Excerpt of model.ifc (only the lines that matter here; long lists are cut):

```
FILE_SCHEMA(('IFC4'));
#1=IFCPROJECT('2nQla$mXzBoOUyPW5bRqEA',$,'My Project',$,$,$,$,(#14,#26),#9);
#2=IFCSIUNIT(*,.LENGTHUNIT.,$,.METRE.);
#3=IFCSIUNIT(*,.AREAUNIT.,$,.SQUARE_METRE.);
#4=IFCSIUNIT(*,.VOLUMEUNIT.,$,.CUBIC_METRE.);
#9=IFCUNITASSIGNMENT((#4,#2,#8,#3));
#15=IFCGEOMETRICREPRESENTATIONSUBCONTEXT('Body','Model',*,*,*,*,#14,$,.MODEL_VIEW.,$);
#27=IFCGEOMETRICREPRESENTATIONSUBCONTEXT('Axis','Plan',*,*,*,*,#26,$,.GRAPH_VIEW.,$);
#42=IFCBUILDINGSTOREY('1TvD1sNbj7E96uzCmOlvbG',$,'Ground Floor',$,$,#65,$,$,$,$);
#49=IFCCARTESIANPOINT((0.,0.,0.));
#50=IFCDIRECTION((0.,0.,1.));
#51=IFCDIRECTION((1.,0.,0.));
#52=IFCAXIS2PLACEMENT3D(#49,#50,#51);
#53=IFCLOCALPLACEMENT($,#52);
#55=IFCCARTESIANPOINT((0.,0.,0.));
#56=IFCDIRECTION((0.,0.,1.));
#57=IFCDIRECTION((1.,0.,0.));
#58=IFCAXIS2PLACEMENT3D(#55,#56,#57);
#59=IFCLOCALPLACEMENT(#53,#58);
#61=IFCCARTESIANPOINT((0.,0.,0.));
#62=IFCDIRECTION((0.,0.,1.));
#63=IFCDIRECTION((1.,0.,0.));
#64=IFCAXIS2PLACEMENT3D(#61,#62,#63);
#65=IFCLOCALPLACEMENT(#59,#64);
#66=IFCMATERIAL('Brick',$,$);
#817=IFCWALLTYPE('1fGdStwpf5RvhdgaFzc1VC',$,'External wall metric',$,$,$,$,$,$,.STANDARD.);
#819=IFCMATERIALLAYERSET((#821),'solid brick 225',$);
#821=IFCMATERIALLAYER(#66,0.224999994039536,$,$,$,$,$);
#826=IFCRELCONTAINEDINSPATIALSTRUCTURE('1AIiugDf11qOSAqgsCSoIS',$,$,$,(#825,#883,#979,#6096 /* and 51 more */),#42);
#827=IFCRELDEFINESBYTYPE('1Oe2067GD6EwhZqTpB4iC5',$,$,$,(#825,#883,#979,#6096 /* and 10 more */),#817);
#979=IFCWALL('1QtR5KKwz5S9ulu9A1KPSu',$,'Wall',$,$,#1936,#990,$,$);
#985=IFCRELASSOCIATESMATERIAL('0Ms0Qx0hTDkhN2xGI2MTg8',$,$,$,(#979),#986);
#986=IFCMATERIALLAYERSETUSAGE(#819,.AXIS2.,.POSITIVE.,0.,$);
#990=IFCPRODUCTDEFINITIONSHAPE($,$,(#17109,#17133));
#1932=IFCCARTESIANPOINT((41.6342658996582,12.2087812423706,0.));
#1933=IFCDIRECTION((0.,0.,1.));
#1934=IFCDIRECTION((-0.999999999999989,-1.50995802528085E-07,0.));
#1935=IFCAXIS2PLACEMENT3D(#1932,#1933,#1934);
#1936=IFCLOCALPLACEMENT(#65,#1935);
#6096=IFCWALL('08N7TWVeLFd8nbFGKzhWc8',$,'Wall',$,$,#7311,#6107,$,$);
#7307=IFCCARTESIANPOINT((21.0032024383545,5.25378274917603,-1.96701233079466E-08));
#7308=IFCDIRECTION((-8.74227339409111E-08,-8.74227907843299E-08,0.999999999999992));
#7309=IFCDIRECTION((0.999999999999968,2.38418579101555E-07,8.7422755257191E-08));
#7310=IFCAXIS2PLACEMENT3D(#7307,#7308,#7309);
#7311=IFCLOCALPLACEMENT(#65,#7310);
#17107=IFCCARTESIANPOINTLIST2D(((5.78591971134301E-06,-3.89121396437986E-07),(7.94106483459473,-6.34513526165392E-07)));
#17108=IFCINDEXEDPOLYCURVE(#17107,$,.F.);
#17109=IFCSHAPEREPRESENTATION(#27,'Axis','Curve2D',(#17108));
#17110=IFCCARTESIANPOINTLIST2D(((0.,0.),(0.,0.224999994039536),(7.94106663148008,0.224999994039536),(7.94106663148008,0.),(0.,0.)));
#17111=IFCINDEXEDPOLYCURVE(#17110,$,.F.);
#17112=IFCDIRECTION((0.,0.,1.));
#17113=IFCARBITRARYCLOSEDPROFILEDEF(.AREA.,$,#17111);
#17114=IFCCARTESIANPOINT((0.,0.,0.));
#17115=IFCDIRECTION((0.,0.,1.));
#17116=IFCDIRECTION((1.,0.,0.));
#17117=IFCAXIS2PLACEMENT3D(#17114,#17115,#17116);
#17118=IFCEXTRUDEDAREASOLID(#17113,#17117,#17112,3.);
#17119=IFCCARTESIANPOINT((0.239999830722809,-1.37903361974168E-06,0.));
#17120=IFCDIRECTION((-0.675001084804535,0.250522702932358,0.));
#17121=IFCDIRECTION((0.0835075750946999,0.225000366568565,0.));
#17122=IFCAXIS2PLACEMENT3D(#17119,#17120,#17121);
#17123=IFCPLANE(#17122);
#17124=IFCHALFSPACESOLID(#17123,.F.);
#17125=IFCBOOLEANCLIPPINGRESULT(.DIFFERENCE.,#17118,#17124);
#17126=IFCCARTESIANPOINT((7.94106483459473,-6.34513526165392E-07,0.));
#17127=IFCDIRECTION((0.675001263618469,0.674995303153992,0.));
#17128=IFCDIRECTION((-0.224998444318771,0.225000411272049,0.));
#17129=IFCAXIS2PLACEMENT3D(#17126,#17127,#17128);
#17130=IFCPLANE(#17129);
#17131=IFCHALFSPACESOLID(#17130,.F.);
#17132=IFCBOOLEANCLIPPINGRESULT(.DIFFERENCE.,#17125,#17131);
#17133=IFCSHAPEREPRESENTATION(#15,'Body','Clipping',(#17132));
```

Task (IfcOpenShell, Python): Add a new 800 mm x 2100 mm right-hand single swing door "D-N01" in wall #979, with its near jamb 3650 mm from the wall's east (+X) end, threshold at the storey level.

```python
import numpy as np
import ifcopenshell
import ifcopenshell.api.feature
import ifcopenshell.api.geometry
import ifcopenshell.api.root
import ifcopenshell.api.spatial
import ifcopenshell.geom
import ifcopenshell.util.element
import ifcopenshell.util.placement
import ifcopenshell.util.representation
import ifcopenshell.util.shape
import ifcopenshell.util.unit

model = ifcopenshell.open("model.ifc")
unit_scale = ifcopenshell.util.unit.calculate_unit_scale(model)
settings = ifcopenshell.geom.settings()


def volume(element):
    """Net volume in cubic metres, openings subtracted."""
    shape = ifcopenshell.geom.create_shape(settings, element)
    return ifcopenshell.util.shape.get_volume(shape.geometry)


wall = model.by_guid("1QtR5KKwz5S9ulu9A1KPSu")
storey = ifcopenshell.util.element.get_container(wall, ifc_class="IfcBuildingStorey")
context = ifcopenshell.util.representation.get_context(model, "Model", "Body", "MODEL_VIEW")
before = volume(wall)

width, height, from_end, sill = 0.8, 2.1, 3.65, 0.0  # metres

# The wall runs along its own X axis, and the end named is its -X end.
wall_shape = ifcopenshell.geom.create_shape(settings, wall)
x, y, z = ifcopenshell.util.shape.get_vertices(wall_shape.geometry).T
start = x.min() + from_end
face, thickness = float(y.min()), float(y.max() - y.min())
wall_matrix = ifcopenshell.util.placement.get_local_placement(wall.ObjectPlacement)
level = ifcopenshell.util.placement.get_local_placement(storey.ObjectPlacement)[2, 3]


def in_wall(x, y):
    """Placement at x, y metres in the wall's axes, at sill height."""
    matrix = wall_matrix.copy()
    matrix[:, 3] = wall_matrix @ np.array([x / unit_scale, y / unit_scale, 0.0, 1.0])
    matrix[2, 3] = level + sill / unit_scale
    return matrix


# Opening: a box that overshoots both wall faces by 50 mm.
opening = ifcopenshell.api.root.create_entity(model, ifc_class="IfcOpeningElement", predefined_type="OPENING")
box = ifcopenshell.api.geometry.add_wall_representation(
    model, context=context, length=width, height=height, thickness=thickness + 0.1
)
ifcopenshell.api.geometry.assign_representation(model, product=opening, representation=box)
ifcopenshell.api.geometry.edit_object_placement(model, product=opening, matrix=in_wall(start, face - 0.05), is_si=False)
ifcopenshell.api.feature.add_feature(model, feature=opening, element=wall)

door = ifcopenshell.api.root.create_entity(model, ifc_class="IfcDoor", name="D-N01", predefined_type="DOOR")
door.OverallWidth, door.OverallHeight = width / unit_scale, height / unit_scale
door.OperationType = "SINGLE_SWING_RIGHT"
body = ifcopenshell.api.geometry.add_door_representation(
    model,
    context=context,
    overall_width=door.OverallWidth,
    overall_height=door.OverallHeight,
    operation_type="SINGLE_SWING_RIGHT",
    lining_properties={"LiningDepth": thickness / unit_scale, "ThresholdDepth": thickness / unit_scale},
)
ifcopenshell.api.geometry.assign_representation(model, product=door, representation=body)
ifcopenshell.api.spatial.assign_container(model, products=[door], relating_structure=storey)
ifcopenshell.api.feature.add_filling(model, opening=opening, element=door)

# The lining spans the wall, so the door starts at the wall face.
ifcopenshell.api.geometry.edit_object_placement(model, product=door, matrix=in_wall(start, face), is_si=False)

after = volume(wall)

print(f"wall volume {before:.3f} -> {after:.3f} m3")

model.write("model_rev.ifc")
```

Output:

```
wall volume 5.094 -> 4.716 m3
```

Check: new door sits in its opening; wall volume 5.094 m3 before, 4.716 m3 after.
